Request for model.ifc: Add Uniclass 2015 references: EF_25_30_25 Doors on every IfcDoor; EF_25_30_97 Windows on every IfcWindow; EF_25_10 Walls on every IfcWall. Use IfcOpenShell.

First a look at what the model holds.

```python
import ifcopenshell

model = ifcopenshell.open("model.ifc")
print(model.schema)
print("classifications:", [c.Name for c in model.by_type("IfcClassification")])
for ifc_class in ("IfcDoor", "IfcRoof", "IfcStair", "IfcWall", "IfcWindow"):
    print(ifc_class, len(model.by_type(ifc_class)))
```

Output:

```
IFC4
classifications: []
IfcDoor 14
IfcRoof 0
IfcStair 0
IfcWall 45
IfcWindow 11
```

```python
import ifcopenshell
import ifcopenshell.api.classification

model = ifcopenshell.open("model.ifc")

system = ifcopenshell.api.classification.add_classification(model, classification="Uniclass 2015")

codes = {
    "IfcDoor": ("EF_25_30_25", "Doors"),
    "IfcWindow": ("EF_25_30_97", "Windows"),
    "IfcWall": ("EF_25_10", "Walls"),
}
for ifc_class, (code, name) in codes.items():
    products = model.by_type(ifc_class)
    ifcopenshell.api.classification.add_reference(
        model, products=products, classification=system, identification=code, name=name
    )
    print(code, len(products))

model.write("model_v2.ifc")
```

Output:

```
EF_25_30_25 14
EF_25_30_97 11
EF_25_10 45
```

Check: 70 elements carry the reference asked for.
